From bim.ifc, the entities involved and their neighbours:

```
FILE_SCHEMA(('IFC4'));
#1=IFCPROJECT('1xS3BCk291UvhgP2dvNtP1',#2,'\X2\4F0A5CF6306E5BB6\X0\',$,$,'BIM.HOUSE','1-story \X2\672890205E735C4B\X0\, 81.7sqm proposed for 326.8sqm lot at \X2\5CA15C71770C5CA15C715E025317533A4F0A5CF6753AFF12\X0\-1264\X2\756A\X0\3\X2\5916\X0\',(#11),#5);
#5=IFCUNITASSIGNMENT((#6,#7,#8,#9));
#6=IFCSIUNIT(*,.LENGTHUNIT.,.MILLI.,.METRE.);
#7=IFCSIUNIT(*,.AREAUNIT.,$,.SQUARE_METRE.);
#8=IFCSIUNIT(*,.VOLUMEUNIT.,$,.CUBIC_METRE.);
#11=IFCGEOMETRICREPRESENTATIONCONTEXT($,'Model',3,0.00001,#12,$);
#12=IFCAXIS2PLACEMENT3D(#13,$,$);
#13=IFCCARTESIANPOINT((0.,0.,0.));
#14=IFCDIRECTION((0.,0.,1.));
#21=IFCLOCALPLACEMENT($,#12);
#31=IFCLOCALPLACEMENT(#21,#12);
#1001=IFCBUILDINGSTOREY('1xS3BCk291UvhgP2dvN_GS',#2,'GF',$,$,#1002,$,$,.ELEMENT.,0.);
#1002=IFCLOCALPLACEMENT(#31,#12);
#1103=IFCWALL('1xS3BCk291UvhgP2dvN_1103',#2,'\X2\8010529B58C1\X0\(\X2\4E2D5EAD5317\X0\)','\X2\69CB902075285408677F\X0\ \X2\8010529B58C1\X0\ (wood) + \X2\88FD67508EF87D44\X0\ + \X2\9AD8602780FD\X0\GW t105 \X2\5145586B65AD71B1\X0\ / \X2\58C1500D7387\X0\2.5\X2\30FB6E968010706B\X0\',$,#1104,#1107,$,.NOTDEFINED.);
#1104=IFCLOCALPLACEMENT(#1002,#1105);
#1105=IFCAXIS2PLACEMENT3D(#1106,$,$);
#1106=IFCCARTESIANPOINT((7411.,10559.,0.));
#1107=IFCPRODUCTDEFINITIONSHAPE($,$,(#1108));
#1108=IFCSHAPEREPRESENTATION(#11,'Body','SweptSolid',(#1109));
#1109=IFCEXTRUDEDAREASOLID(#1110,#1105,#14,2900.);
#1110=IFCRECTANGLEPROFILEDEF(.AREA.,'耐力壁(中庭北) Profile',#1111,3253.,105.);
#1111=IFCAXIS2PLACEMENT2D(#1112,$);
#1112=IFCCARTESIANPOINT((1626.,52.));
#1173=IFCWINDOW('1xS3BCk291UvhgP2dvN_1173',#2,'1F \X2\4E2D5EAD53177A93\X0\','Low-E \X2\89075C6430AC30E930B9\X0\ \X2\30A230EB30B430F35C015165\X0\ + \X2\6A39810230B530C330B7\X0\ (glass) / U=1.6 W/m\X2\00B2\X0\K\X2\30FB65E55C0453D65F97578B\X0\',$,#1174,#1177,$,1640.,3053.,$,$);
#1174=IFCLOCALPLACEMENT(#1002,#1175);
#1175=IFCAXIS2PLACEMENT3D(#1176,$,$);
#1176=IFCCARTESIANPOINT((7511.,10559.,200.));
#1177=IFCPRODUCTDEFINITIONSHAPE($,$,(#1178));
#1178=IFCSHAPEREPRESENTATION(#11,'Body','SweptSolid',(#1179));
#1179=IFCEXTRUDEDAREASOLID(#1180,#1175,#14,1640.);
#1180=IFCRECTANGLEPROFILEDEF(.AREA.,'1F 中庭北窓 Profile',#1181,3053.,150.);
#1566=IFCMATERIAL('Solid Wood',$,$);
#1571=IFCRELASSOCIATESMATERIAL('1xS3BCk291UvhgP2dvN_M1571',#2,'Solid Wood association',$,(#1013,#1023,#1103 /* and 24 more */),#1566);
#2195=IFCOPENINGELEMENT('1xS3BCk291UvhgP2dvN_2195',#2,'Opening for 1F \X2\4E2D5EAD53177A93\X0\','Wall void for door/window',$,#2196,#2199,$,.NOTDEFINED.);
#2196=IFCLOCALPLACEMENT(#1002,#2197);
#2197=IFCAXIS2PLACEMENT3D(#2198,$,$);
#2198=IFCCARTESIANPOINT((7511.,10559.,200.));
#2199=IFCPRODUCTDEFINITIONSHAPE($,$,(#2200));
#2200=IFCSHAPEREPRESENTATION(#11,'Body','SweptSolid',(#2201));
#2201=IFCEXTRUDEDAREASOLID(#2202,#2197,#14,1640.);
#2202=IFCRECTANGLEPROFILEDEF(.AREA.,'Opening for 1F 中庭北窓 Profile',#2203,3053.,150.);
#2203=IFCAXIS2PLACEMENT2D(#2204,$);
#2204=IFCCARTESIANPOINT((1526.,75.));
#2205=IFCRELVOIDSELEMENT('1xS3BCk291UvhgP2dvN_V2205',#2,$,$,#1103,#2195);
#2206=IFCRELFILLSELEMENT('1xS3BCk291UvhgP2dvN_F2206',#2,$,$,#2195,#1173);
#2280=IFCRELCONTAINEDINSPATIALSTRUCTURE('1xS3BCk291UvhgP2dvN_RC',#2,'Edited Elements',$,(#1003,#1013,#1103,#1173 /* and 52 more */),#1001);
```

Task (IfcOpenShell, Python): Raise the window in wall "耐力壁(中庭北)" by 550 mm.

```python
import numpy as np
import ifcopenshell
import ifcopenshell.api.geometry
import ifcopenshell.util.placement
import ifcopenshell.util.unit

model = ifcopenshell.open("bim.ifc")
unit_scale = ifcopenshell.util.unit.calculate_unit_scale(model)

window = model.by_guid("1xS3BCk291UvhgP2dvN_1173")
opening = window.FillsVoids[0].RelatingOpeningElement
dz = 0.55 / unit_scale

shift = np.array([0.0, 0.0, dz])
# The window is not placed relative to its opening, so move both.
for product in (opening, window):
    matrix = ifcopenshell.util.placement.get_local_placement(product.ObjectPlacement)
    matrix[:3, 3] += shift
    ifcopenshell.api.geometry.edit_object_placement(model, product=product, matrix=matrix, is_si=False)

print(f"moved by {dz * unit_scale:+.3f} m")

model.write("bim_edited.ifc")
```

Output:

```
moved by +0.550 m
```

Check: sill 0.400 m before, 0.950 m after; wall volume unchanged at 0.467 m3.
